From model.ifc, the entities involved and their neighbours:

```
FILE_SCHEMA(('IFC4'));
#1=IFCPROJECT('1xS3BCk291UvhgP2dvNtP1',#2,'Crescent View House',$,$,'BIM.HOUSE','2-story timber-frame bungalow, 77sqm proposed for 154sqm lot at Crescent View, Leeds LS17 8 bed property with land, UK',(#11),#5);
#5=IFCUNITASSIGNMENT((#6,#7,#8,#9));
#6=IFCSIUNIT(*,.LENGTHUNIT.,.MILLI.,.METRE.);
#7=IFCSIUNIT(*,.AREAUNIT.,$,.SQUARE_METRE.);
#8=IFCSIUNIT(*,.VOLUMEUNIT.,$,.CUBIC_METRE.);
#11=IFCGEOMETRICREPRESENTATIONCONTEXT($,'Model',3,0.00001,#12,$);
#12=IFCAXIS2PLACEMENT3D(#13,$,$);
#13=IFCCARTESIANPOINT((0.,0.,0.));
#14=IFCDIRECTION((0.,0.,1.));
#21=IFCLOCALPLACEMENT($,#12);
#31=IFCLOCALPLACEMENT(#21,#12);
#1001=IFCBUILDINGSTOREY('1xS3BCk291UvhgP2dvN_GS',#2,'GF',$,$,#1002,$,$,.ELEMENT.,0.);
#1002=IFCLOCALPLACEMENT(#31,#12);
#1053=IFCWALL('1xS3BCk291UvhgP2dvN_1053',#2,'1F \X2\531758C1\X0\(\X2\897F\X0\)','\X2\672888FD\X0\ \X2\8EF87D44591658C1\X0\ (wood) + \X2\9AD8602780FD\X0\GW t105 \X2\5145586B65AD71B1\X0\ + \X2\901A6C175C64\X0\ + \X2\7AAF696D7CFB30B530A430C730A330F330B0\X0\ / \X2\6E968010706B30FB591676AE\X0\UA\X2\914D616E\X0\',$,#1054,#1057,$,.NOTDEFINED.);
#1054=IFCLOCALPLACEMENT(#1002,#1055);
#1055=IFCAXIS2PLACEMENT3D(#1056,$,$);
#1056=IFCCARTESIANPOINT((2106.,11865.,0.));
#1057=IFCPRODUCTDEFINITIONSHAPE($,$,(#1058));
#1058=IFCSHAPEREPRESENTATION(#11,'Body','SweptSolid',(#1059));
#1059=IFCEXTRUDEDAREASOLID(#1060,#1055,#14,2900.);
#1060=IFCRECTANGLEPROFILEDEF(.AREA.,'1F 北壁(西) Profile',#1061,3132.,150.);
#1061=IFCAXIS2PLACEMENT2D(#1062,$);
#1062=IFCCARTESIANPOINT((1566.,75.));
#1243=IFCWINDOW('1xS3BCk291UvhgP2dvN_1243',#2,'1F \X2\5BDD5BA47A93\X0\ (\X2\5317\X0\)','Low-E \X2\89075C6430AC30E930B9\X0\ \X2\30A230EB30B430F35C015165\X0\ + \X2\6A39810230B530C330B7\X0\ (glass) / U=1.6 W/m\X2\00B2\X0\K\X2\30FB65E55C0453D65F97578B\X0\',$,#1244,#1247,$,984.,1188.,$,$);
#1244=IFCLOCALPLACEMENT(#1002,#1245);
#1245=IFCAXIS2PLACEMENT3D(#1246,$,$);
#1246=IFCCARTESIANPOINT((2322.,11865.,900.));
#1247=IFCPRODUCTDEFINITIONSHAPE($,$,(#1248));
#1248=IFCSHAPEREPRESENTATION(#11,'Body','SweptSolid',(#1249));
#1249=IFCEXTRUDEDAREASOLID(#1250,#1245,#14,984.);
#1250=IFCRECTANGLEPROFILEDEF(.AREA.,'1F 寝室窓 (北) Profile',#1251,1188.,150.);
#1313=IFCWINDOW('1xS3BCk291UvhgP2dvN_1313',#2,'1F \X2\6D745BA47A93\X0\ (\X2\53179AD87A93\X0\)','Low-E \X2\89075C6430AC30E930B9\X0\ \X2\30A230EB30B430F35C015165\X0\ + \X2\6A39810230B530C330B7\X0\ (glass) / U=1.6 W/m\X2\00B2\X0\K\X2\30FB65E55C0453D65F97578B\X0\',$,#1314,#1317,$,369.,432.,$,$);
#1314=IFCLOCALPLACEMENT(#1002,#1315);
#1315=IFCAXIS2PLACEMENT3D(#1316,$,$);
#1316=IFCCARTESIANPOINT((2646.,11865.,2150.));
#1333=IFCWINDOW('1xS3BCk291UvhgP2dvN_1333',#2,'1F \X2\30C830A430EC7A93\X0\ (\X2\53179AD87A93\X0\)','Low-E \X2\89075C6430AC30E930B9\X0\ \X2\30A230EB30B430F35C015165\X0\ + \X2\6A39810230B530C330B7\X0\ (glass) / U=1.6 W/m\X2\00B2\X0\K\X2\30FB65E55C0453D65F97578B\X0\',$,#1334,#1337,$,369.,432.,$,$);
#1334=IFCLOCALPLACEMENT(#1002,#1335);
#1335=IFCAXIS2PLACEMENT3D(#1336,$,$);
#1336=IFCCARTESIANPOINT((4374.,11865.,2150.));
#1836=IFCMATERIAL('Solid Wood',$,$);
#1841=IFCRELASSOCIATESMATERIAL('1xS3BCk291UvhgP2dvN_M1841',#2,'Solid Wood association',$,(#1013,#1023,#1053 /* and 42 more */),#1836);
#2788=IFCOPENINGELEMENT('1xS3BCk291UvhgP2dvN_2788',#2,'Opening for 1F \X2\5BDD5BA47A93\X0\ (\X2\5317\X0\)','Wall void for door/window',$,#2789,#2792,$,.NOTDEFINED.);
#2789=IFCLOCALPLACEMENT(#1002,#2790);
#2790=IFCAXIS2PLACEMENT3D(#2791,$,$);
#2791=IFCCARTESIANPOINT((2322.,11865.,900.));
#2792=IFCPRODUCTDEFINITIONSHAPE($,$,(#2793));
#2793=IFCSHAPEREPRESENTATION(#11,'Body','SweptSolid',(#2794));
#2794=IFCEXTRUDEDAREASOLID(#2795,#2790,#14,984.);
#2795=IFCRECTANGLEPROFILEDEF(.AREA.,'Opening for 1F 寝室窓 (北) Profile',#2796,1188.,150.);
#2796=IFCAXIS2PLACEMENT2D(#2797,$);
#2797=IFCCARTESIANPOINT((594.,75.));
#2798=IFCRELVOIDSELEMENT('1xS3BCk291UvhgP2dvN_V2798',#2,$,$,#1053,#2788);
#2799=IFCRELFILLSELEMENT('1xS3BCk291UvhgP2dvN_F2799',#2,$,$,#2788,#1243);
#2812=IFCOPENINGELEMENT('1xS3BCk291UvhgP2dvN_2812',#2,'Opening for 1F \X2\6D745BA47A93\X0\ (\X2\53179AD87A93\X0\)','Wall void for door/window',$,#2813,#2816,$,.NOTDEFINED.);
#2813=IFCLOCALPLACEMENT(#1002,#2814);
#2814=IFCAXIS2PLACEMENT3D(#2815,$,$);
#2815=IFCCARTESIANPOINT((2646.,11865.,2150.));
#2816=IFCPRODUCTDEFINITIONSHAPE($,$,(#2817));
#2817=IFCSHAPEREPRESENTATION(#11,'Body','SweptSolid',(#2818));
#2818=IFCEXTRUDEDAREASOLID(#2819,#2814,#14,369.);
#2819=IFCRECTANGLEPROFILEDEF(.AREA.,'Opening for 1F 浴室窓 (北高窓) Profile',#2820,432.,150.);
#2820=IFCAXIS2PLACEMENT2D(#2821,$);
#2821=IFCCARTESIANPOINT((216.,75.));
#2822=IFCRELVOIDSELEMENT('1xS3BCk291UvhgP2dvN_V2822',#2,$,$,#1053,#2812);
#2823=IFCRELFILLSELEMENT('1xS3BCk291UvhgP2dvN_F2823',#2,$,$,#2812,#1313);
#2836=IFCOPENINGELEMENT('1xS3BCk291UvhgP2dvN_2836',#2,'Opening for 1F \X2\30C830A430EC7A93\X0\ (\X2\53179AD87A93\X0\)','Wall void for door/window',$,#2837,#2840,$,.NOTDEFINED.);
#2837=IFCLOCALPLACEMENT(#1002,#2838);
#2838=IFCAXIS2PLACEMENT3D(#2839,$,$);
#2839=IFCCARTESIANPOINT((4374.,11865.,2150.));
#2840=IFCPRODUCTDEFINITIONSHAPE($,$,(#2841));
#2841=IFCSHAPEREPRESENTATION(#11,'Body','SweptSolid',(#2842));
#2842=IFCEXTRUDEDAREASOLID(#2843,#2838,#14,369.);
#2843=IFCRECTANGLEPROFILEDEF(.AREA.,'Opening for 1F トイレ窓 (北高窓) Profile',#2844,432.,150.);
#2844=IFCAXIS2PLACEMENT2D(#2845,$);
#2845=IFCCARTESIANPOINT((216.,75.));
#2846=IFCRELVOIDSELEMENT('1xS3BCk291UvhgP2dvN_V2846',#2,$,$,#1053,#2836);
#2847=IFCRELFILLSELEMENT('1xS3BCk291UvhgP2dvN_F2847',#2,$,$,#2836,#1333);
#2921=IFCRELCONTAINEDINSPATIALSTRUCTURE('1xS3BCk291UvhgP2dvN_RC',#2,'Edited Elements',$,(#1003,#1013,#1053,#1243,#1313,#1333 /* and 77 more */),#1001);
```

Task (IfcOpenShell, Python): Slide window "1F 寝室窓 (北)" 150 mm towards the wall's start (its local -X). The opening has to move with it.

```python
import ifcopenshell
import ifcopenshell.api.geometry
import ifcopenshell.util.placement

model = ifcopenshell.open("model.ifc")

window = model.by_guid("1xS3BCk291UvhgP2dvN_1243")
opening = window.FillsVoids[0].RelatingOpeningElement
wall = opening.VoidsElements[0].RelatingBuildingElement

wall_matrix = ifcopenshell.util.placement.get_local_placement(wall.ObjectPlacement)
shift = wall_matrix[:3, 0] * -150.0
before = ifcopenshell.util.placement.get_local_placement(window.ObjectPlacement)[:3, 3].copy()

# The window is not placed relative to its opening, so move both.
for product in (opening, window):
    matrix = ifcopenshell.util.placement.get_local_placement(product.ObjectPlacement)
    matrix[:3, 3] += shift
    ifcopenshell.api.geometry.edit_object_placement(model, product=product, matrix=matrix, is_si=False)

after = ifcopenshell.util.placement.get_local_placement(window.ObjectPlacement)[:3, 3]
print("window moved by", (after - before).round(3) + 0.0)

model.write("model-out.ifc")
```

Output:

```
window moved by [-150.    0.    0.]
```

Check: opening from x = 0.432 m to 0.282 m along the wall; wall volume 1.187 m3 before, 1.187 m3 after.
